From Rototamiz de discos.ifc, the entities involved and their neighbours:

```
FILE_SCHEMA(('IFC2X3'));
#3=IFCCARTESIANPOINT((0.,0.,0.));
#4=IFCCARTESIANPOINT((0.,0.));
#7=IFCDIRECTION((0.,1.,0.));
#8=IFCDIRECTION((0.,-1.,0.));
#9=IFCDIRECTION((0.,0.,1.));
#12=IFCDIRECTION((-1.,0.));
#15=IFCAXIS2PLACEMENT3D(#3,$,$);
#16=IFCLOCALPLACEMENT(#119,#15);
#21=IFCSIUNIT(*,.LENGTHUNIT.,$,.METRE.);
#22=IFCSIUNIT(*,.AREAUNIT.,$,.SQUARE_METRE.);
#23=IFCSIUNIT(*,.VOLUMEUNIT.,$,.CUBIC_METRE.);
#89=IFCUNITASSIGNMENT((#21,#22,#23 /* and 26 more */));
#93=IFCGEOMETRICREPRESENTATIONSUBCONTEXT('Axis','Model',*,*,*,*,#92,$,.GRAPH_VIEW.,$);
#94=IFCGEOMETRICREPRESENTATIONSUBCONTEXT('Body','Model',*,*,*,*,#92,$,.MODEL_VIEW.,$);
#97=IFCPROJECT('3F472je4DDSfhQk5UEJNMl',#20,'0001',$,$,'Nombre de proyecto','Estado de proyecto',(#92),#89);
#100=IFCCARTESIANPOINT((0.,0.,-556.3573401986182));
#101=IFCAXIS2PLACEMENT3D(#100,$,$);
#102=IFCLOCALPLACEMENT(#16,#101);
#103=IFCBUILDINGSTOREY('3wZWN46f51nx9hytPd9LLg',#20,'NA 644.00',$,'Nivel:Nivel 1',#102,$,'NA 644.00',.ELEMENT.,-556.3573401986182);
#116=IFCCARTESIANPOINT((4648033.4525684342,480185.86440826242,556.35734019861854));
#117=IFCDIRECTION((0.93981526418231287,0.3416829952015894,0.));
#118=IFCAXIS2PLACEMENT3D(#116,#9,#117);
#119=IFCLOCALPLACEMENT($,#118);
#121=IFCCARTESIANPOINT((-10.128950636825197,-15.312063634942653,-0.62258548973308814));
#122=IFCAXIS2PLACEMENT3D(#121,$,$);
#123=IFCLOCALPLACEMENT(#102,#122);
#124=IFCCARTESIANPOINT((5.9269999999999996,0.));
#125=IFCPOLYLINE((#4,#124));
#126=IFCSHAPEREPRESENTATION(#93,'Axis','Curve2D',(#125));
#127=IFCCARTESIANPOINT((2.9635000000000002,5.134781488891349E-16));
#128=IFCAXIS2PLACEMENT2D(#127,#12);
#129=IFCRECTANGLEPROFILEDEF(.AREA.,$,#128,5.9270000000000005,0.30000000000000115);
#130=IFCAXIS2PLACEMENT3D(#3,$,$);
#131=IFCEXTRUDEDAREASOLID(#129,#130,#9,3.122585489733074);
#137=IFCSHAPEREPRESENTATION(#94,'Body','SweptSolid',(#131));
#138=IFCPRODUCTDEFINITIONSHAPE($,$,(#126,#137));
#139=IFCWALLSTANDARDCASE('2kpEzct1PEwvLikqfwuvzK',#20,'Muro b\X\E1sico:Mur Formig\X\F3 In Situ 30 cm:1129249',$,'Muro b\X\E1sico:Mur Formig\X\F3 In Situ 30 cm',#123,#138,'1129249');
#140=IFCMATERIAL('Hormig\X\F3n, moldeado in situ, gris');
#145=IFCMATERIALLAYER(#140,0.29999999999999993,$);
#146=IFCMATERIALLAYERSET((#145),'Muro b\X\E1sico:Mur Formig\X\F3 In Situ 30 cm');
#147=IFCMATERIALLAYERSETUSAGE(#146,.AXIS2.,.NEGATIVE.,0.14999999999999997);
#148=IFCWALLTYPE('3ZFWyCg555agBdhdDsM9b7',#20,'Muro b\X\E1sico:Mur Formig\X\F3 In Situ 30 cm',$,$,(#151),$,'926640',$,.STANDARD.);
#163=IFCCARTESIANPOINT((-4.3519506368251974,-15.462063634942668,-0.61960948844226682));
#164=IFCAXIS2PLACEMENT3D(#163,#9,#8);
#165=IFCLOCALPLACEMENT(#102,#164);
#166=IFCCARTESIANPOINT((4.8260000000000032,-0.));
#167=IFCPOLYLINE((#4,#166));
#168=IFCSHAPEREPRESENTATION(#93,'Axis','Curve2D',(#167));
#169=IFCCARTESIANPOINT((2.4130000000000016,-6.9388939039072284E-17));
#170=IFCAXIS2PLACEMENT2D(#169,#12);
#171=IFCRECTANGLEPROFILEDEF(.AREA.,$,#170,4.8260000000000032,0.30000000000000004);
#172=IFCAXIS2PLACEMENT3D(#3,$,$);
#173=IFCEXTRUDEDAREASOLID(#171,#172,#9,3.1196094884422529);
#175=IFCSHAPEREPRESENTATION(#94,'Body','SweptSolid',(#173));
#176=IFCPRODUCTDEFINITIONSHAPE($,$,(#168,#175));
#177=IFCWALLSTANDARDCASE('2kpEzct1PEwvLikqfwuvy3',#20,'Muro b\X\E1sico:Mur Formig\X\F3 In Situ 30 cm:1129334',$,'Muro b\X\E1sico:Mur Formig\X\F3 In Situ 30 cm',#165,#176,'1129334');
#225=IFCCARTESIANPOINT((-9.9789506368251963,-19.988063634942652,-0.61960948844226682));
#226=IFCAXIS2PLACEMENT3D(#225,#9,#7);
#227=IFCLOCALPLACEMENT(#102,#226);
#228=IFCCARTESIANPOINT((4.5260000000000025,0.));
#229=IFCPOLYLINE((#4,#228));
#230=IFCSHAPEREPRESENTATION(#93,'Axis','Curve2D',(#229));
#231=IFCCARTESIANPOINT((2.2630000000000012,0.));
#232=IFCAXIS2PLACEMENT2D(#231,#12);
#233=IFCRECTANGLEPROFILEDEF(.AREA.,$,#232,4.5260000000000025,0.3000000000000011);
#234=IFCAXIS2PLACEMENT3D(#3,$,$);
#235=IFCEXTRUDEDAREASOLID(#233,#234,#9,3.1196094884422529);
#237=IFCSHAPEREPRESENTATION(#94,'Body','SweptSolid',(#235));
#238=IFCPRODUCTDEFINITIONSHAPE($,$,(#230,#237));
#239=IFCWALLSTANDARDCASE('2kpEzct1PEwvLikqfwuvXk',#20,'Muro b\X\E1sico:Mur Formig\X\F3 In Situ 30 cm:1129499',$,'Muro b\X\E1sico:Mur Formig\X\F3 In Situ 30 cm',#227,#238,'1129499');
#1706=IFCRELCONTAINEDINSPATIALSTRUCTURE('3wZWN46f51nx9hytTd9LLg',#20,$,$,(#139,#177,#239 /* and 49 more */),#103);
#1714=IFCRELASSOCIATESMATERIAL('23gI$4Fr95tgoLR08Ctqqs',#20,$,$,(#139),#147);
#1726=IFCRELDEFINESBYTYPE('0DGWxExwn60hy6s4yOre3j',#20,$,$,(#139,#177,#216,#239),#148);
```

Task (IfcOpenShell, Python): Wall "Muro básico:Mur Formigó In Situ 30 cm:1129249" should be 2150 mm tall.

```python
import ifcopenshell
import ifcopenshell.geom
import ifcopenshell.util.representation
import ifcopenshell.util.shape

model = ifcopenshell.open("Rototamiz de discos.ifc")
settings = ifcopenshell.geom.settings()


def volume(element):
    """Net volume in cubic metres, openings subtracted."""
    shape = ifcopenshell.geom.create_shape(settings, element)
    return ifcopenshell.util.shape.get_volume(shape.geometry)


wall = model.by_guid("2kpEzct1PEwvLikqfwuvzK")
before = volume(wall)

body = ifcopenshell.util.representation.get_representation(wall, "Model", "Body")
solid = body.Items[0]
old_height = solid.Depth
solid.Depth = 2.15
after = volume(wall)

print(f"height {old_height:g} -> {solid.Depth:g}, volume {before:.3f} -> {after:.3f} m3")

model.write("Rototamiz de discos_rev.ifc")
```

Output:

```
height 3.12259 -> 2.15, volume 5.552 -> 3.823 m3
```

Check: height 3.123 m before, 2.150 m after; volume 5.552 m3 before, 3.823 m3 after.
